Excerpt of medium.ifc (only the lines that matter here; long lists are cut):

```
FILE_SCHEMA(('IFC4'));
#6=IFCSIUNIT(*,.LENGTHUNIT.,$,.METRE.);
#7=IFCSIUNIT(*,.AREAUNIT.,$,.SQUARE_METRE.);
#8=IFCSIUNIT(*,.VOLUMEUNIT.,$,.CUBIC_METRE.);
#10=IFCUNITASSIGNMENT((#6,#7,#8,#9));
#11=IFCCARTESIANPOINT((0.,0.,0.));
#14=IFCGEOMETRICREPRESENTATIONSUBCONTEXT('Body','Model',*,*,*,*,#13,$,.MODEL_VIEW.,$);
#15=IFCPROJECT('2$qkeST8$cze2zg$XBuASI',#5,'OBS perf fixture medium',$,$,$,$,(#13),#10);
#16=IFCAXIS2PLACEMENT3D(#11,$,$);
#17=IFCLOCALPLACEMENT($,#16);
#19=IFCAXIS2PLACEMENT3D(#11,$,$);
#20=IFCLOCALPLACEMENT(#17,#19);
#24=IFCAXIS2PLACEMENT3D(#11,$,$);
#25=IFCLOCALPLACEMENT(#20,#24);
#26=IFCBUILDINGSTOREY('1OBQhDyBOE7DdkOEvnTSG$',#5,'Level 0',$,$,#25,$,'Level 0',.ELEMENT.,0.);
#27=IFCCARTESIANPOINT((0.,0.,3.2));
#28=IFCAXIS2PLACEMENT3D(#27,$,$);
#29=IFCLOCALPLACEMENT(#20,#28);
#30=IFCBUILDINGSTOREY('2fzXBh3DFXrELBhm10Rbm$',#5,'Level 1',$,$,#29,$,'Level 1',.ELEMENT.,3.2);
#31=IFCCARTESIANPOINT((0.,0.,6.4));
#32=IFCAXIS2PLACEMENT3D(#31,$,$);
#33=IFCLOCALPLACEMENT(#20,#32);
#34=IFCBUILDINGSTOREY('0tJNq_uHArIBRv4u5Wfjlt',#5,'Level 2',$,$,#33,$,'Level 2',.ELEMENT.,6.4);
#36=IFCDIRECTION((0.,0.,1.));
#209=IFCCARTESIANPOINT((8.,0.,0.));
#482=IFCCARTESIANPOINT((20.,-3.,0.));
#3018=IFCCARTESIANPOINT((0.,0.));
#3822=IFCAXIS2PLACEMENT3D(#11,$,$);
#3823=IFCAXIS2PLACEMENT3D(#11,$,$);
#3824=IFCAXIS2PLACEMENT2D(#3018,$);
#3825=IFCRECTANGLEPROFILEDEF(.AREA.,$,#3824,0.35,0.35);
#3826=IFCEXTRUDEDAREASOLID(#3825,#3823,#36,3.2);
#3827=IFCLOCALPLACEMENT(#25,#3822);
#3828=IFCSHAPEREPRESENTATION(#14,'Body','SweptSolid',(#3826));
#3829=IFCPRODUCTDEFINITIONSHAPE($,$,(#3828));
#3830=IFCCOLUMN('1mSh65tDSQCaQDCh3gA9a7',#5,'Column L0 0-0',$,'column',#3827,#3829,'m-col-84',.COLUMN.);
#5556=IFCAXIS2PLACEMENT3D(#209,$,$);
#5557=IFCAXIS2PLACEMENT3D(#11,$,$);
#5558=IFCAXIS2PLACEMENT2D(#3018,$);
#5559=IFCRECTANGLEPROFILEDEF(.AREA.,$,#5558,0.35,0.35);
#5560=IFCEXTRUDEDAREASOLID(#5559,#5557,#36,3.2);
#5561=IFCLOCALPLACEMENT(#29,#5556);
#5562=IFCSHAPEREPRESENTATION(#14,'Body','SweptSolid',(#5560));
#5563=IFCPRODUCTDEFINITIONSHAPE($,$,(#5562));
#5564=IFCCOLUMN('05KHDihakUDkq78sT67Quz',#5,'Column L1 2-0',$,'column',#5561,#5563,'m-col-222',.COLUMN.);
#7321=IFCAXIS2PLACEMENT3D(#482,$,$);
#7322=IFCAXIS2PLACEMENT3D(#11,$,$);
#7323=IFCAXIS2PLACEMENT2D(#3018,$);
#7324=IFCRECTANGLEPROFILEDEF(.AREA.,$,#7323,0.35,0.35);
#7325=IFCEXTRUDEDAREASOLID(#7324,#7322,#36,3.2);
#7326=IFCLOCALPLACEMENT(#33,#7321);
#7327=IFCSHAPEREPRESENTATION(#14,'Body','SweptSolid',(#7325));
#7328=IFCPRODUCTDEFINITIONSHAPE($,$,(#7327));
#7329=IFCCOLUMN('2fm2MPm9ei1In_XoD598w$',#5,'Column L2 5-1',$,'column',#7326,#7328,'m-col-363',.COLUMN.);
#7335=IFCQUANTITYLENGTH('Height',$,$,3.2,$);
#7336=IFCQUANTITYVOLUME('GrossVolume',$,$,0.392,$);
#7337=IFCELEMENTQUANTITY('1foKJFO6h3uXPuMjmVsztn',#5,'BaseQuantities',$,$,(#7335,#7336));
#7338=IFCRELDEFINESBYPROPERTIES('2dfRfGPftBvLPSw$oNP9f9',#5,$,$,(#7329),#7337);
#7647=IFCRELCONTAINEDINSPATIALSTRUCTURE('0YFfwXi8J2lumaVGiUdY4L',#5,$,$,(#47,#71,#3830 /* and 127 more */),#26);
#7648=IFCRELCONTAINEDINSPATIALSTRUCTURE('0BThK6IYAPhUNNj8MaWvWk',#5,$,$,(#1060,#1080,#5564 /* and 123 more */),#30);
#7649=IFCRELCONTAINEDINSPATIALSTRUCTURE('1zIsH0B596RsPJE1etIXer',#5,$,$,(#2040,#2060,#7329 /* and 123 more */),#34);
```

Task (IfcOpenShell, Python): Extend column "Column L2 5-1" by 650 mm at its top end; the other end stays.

```python
import ifcopenshell
import ifcopenshell.api.pset
import ifcopenshell.util.element
import ifcopenshell.util.representation
import ifcopenshell.util.unit

model = ifcopenshell.open("medium.ifc")
unit_scale = ifcopenshell.util.unit.calculate_unit_scale(model)

member = model.by_guid("2fm2MPm9ei1In_XoD598w$")
change = 0.65 / unit_scale

# The extrusion runs towards the end named, so only its depth changes.
body = ifcopenshell.util.representation.get_representation(member, "Model", "Body")
solid = body.Items[0]
old_length = solid.Depth
solid.Depth += change

# Update the stored length and volume.
qto = model.by_id(ifcopenshell.util.element.get_pset(member, "BaseQuantities", should_inherit=False)["id"])
ifcopenshell.api.pset.edit_qto(model, qto=qto, properties={
    "Height": solid.Depth,
    "GrossVolume": ifcopenshell.util.element.get_pset(member, "BaseQuantities", "GrossVolume") * solid.Depth / old_length,
})

print(f"length {old_length:g} -> {solid.Depth:g}")

model.write("medium-out.ifc")
```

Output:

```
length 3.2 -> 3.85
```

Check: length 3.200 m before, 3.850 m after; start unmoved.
